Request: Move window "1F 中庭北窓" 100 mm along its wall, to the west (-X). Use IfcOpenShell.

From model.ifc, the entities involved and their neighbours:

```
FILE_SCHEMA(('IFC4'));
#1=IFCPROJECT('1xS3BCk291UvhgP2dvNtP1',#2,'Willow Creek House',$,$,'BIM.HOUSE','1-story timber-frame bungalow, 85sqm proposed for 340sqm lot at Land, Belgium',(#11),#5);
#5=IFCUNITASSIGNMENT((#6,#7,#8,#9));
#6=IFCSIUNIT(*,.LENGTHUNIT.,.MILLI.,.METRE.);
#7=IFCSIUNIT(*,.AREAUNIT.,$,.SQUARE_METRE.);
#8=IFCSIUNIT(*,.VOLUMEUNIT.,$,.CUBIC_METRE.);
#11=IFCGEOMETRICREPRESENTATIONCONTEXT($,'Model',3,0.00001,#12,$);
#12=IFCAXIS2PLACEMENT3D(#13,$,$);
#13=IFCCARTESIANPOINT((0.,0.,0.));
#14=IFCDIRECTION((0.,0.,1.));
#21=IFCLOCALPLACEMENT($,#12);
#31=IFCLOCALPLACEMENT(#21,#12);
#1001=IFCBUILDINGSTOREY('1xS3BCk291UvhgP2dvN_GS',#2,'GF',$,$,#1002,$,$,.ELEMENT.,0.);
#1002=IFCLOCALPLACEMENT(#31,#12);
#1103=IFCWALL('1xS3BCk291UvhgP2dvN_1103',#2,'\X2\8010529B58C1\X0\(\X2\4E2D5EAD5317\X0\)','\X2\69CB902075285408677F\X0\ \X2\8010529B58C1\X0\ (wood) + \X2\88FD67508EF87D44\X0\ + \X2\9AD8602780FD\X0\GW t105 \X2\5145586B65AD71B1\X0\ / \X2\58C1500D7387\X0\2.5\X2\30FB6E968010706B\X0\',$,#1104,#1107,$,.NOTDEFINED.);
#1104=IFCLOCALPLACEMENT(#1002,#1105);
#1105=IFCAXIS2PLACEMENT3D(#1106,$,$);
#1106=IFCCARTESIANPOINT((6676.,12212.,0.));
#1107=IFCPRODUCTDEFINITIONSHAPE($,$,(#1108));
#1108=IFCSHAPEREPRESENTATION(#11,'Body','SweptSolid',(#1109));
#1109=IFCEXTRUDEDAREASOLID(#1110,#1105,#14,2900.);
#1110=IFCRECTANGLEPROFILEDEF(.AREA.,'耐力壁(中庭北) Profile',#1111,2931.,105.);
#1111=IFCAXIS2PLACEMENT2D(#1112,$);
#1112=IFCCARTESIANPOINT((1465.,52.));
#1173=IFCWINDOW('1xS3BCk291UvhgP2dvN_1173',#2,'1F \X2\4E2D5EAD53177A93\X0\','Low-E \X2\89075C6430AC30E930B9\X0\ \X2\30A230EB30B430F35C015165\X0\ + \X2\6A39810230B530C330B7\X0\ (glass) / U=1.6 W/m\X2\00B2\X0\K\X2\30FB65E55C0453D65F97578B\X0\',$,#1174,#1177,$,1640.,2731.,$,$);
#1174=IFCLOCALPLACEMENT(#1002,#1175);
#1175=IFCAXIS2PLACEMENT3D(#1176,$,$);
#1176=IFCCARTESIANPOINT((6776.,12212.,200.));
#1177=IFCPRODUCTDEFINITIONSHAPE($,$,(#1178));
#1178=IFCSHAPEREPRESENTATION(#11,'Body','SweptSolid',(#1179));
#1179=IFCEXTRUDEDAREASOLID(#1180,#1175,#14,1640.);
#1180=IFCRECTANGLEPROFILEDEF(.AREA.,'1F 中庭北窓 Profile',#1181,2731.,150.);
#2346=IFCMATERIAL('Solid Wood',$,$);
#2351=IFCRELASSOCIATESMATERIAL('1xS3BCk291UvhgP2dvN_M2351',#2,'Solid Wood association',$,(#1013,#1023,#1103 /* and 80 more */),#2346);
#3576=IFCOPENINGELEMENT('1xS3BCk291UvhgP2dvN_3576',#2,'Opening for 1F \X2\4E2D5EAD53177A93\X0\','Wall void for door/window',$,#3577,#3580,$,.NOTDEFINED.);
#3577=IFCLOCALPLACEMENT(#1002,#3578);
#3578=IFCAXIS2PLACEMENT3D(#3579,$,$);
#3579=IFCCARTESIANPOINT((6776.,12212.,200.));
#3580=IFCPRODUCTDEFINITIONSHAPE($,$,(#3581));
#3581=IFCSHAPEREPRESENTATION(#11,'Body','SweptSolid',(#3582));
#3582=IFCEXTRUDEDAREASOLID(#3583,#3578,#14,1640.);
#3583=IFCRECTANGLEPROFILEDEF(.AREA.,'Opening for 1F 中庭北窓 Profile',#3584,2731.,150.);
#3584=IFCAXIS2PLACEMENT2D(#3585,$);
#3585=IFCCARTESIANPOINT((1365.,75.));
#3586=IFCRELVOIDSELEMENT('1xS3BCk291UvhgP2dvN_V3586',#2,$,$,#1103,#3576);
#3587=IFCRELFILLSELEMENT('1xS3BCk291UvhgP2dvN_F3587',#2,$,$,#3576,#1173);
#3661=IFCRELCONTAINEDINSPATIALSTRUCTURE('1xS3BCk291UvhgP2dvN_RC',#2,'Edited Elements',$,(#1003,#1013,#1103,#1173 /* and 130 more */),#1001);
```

```python
import ifcopenshell
import ifcopenshell.api.geometry
import ifcopenshell.util.placement
import ifcopenshell.util.unit

model = ifcopenshell.open("model.ifc")
unit_scale = ifcopenshell.util.unit.calculate_unit_scale(model)

window = model.by_guid("1xS3BCk291UvhgP2dvN_1173")
opening = window.FillsVoids[0].RelatingOpeningElement
wall = opening.VoidsElements[0].RelatingBuildingElement

wall_matrix = ifcopenshell.util.placement.get_local_placement(wall.ObjectPlacement)
shift = wall_matrix[:3, 0] * -0.1 / unit_scale
before = ifcopenshell.util.placement.get_local_placement(window.ObjectPlacement)[:3, 3].copy()

# The window is not placed relative to its opening, so move both.
for product in (opening, window):
    matrix = ifcopenshell.util.placement.get_local_placement(product.ObjectPlacement)
    matrix[:3, 3] += shift
    ifcopenshell.api.geometry.edit_object_placement(model, product=product, matrix=matrix, is_si=False)

after = ifcopenshell.util.placement.get_local_placement(window.ObjectPlacement)[:3, 3]
print("window moved by", (after - before).round(3) + 0.0)

model.write("model_updated.ifc")
```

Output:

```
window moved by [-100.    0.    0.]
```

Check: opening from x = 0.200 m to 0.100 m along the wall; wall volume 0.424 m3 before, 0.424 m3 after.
